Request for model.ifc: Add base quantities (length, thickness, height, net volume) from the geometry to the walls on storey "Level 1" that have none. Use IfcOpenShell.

First a look at what the model holds.

```python
import ifcopenshell
import ifcopenshell.util.element
import ifcopenshell.util.unit

model = ifcopenshell.open("model.ifc")
print(model.schema)
for unit_type in ("LENGTHUNIT", "AREAUNIT", "VOLUMEUNIT"):
    print(unit_type, ifcopenshell.util.unit.calculate_unit_scale(model, unit_type))
storey = next(s for s in model.by_type("IfcBuildingStorey") if s.Name == "Level 1")
walls = [e for e in ifcopenshell.util.element.get_decomposition(storey) if e.is_a("IfcWall")]
for e in sorted(walls, key=lambda e: e.id()):
    print(e.id(), e.is_a(), e.Name, list(ifcopenshell.util.element.get_psets(e, qtos_only=True)), sep=" | ")
```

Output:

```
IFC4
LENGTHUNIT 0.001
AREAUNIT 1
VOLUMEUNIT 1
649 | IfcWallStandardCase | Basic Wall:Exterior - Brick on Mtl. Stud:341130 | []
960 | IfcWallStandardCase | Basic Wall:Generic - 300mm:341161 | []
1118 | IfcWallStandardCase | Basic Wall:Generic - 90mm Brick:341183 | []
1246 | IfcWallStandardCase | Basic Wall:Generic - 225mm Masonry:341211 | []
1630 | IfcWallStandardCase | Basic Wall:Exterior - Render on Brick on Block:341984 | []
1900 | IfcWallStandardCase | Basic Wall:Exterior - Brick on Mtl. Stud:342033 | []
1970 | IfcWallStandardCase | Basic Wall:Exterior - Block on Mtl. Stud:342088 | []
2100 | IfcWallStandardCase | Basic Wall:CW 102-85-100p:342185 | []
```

```python
import ifcopenshell
import ifcopenshell.api.pset
import ifcopenshell.geom
import ifcopenshell.util.element
import ifcopenshell.util.shape
import ifcopenshell.util.unit

model = ifcopenshell.open("model.ifc")
unit_scale = ifcopenshell.util.unit.calculate_unit_scale(model)
volume_scale = ifcopenshell.util.unit.calculate_unit_scale(model, "VOLUMEUNIT")
settings = ifcopenshell.geom.settings()

storey = next(s for s in model.by_type("IfcBuildingStorey") if s.Name == "Level 1")
walls = [e for e in ifcopenshell.util.element.get_decomposition(storey) if e.is_a("IfcWall")]

for e in sorted(walls, key=lambda e: e.id()):
    if ifcopenshell.util.element.get_psets(e, qtos_only=True, should_inherit=False):
        continue
    # Geometry comes back in metres, in the element's own axes.
    shape = ifcopenshell.geom.create_shape(settings, e)
    values = {
        "Length": ifcopenshell.util.shape.get_x(shape.geometry) / unit_scale,
        "Width": ifcopenshell.util.shape.get_y(shape.geometry) / unit_scale,
        "Height": ifcopenshell.util.shape.get_z(shape.geometry) / unit_scale,
        "NetVolume": ifcopenshell.util.shape.get_volume(shape.geometry) / volume_scale,
    }
    qto = ifcopenshell.api.pset.add_qto(model, product=e, name="Qto_WallBaseQuantities")
    ifcopenshell.api.pset.edit_qto(model, qto=qto, properties=values)
    print(e.id(), {k: round(v, 3) for k, v in values.items()})

model.write("model_updated.ifc")
```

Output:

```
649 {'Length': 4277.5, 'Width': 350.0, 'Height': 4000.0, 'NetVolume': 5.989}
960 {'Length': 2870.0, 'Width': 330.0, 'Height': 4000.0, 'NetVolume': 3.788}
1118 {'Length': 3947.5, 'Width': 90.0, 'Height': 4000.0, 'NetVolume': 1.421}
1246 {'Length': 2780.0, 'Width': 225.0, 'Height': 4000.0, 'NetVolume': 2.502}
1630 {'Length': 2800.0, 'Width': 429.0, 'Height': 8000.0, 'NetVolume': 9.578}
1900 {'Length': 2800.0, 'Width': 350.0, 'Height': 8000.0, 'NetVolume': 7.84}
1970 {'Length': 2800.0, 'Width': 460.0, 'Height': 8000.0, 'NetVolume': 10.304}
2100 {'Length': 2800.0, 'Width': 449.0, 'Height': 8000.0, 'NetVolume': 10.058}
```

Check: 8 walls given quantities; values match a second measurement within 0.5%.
